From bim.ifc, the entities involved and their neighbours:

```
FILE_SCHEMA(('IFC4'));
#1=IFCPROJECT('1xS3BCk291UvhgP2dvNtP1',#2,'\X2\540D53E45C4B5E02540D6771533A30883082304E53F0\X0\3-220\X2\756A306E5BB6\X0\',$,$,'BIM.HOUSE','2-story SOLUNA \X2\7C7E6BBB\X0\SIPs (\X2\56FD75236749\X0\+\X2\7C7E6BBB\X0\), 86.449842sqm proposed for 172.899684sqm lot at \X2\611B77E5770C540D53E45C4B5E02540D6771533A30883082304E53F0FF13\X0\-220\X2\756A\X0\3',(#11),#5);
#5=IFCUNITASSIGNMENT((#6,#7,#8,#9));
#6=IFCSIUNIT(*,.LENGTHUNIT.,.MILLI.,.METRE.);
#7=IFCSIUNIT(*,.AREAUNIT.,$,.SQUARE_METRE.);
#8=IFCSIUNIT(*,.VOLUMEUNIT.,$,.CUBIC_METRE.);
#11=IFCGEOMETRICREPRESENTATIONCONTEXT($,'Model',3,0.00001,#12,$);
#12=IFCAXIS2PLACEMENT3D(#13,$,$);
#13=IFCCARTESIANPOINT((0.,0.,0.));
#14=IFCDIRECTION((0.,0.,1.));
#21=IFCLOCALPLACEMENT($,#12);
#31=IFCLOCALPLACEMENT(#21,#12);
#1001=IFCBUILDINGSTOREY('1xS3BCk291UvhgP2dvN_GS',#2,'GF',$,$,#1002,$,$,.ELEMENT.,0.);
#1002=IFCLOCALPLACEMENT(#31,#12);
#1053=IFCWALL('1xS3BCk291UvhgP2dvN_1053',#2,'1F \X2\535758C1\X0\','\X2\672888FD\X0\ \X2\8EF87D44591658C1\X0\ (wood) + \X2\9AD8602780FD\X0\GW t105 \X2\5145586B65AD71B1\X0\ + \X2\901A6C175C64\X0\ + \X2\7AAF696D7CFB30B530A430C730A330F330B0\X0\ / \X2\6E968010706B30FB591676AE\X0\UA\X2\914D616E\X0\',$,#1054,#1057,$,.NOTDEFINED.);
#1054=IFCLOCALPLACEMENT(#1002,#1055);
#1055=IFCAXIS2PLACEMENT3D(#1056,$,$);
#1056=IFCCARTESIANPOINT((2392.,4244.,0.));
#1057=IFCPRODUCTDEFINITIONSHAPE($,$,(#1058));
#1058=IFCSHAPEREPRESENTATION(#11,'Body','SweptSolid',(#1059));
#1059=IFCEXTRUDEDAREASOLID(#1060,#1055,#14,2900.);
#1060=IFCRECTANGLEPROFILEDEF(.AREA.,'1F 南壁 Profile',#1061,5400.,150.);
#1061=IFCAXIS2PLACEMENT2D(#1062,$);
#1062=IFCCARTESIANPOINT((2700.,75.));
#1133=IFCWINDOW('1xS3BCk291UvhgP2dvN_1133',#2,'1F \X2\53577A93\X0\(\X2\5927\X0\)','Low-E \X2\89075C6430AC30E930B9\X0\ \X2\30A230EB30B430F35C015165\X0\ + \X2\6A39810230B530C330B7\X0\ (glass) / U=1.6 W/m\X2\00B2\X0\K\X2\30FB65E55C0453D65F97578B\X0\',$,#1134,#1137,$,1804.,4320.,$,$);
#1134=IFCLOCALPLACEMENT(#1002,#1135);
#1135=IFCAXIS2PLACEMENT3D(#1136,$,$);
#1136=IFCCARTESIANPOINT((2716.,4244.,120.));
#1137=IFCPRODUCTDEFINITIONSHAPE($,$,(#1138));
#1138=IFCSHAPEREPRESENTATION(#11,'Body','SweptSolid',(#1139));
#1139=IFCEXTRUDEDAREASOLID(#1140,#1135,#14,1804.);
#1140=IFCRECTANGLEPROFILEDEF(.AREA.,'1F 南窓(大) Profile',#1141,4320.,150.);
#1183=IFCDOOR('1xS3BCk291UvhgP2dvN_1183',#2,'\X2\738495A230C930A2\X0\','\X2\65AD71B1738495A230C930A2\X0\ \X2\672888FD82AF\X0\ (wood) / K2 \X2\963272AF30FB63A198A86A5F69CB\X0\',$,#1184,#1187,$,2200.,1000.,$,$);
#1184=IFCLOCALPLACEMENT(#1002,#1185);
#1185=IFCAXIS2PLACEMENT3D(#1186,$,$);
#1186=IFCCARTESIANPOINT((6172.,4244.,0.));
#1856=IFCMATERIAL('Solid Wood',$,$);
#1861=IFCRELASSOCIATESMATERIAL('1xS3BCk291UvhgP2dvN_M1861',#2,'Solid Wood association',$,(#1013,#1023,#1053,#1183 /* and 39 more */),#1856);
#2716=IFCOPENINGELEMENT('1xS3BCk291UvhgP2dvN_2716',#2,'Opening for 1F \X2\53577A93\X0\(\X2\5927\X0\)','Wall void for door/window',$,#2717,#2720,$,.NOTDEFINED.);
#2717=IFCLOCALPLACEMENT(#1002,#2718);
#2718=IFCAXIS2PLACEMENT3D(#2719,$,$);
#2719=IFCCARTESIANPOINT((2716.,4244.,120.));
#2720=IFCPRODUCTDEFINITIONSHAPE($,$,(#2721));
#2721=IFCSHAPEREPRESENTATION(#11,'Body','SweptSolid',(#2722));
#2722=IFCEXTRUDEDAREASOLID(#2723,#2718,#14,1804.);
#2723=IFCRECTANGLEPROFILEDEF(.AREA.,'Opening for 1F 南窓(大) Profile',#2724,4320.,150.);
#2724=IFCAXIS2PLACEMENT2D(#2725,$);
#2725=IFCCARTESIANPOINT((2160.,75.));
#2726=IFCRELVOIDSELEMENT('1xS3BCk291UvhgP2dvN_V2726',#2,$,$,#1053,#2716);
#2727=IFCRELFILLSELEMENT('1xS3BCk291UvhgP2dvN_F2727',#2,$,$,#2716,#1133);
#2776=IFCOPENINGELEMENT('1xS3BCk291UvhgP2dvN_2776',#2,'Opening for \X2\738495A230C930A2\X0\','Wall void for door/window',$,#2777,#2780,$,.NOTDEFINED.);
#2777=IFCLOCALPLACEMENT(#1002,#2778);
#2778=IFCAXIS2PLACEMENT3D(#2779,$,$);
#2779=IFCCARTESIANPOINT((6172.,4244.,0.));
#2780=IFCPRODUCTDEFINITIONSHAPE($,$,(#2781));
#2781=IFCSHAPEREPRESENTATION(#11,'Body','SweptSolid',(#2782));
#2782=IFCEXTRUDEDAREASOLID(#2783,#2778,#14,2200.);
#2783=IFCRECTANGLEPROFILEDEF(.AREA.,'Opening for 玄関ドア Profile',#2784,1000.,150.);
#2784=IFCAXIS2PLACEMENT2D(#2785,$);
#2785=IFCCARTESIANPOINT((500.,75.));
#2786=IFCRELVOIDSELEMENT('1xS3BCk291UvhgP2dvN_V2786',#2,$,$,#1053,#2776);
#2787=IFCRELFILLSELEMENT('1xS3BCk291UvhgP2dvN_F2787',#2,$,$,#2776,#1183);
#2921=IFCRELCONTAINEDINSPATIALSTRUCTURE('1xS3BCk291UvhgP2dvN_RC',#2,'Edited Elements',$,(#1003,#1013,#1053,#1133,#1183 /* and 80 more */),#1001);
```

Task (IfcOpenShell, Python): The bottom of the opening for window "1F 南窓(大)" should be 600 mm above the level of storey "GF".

```python
import numpy as np
import ifcopenshell
import ifcopenshell.api.geometry
import ifcopenshell.geom
import ifcopenshell.util.element
import ifcopenshell.util.placement
import ifcopenshell.util.shape
import ifcopenshell.util.unit

model = ifcopenshell.open("bim.ifc")
unit_scale = ifcopenshell.util.unit.calculate_unit_scale(model)

window = model.by_guid("1xS3BCk291UvhgP2dvN_1133")
opening = window.FillsVoids[0].RelatingOpeningElement
storey = ifcopenshell.util.element.get_container(window, ifc_class="IfcBuildingStorey")
level = ifcopenshell.util.placement.get_local_placement(storey.ObjectPlacement)[2, 3]

# The opening's origin need not be at the sill, so measure its lowest point.
shape = ifcopenshell.geom.create_shape(ifcopenshell.geom.settings(), opening)
bottom = ifcopenshell.util.shape.get_shape_bottom_elevation(shape, shape.geometry) / unit_scale
dz = level + 600.0 - bottom

shift = np.array([0.0, 0.0, dz])
# The window is not placed relative to its opening, so move both.
for product in (opening, window):
    matrix = ifcopenshell.util.placement.get_local_placement(product.ObjectPlacement)
    matrix[:3, 3] += shift
    ifcopenshell.api.geometry.edit_object_placement(model, product=product, matrix=matrix, is_si=False)

print(f"moved by {dz * unit_scale:+.3f} m")

model.write("bim-out.ifc")
```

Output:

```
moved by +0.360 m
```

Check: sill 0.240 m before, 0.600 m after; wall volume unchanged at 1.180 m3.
